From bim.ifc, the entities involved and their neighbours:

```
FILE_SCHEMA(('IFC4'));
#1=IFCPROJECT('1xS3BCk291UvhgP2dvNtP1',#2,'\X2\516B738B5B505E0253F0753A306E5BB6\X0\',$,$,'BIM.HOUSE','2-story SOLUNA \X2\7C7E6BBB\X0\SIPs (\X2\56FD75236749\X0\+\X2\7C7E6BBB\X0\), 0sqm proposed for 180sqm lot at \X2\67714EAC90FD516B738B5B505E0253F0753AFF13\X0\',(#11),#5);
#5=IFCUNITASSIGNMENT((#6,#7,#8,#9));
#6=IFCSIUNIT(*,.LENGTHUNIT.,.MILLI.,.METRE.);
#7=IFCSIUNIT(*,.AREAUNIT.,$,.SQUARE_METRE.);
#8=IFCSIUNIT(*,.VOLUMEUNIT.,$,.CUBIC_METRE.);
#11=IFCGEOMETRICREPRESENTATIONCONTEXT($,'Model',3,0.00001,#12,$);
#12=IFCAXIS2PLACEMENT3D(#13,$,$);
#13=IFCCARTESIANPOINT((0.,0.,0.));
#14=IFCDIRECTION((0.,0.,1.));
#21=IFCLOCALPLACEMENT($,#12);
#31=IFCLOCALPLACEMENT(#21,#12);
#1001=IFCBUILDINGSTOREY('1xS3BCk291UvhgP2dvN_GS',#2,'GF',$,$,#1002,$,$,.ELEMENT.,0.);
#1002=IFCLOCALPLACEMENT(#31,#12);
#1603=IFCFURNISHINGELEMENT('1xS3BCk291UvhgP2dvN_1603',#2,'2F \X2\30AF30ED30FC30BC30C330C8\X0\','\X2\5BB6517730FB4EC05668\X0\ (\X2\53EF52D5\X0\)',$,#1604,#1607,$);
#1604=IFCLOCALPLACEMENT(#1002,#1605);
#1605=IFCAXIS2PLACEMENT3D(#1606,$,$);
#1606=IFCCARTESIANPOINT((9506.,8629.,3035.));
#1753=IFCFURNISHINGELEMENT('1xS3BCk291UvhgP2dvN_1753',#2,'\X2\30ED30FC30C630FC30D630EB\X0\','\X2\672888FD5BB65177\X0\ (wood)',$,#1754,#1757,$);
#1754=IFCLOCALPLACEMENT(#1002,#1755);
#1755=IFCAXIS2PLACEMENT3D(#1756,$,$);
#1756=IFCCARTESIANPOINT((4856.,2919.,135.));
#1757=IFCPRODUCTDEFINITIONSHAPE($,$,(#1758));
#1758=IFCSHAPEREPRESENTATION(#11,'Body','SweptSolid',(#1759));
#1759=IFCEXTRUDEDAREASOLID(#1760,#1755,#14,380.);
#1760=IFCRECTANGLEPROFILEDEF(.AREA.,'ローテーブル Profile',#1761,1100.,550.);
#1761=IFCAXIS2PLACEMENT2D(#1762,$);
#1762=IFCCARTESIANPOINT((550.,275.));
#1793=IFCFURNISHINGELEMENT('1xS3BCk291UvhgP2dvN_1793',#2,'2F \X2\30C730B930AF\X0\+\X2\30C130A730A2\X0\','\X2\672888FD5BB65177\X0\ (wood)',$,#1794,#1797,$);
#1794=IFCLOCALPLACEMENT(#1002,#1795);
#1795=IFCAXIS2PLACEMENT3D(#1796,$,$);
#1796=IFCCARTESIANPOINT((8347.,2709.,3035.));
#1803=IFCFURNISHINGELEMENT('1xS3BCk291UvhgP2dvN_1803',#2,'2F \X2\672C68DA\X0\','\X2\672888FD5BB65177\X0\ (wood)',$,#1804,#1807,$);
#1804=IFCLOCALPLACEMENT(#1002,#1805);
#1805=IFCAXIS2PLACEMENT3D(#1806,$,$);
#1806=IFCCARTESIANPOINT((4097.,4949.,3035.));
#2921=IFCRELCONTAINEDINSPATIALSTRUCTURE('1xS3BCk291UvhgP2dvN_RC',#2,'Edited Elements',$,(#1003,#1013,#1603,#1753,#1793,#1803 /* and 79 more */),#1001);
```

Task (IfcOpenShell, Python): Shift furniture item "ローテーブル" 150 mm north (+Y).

```python
import ifcopenshell
import ifcopenshell.api.geometry
import ifcopenshell.util.placement

model = ifcopenshell.open("bim.ifc")

item = model.by_id(1753)
matrix = ifcopenshell.util.placement.get_local_placement(item.ObjectPlacement)
matrix[1, 3] += 150.0
ifcopenshell.api.geometry.edit_object_placement(model, product=item, matrix=matrix, is_si=False)

print(ifcopenshell.util.placement.get_local_placement(item.ObjectPlacement).round(3) + 0.0)

model.write("bim-out.ifc")
```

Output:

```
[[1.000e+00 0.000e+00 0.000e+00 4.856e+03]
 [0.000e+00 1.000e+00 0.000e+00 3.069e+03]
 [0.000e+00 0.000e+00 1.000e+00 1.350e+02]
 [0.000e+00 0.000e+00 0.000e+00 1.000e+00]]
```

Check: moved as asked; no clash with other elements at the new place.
